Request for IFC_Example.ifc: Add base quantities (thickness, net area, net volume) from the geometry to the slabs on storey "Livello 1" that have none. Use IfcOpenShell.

First a look at what the model holds.

```python
import ifcopenshell
import ifcopenshell.util.element
import ifcopenshell.util.unit

model = ifcopenshell.open("IFC_Example.ifc")
print(model.schema)
for unit_type in ("LENGTHUNIT", "AREAUNIT", "VOLUMEUNIT"):
    print(unit_type, ifcopenshell.util.unit.calculate_unit_scale(model, unit_type))
storey = next(s for s in model.by_type("IfcBuildingStorey") if s.Name == "Livello 1")
slabs = [e for e in ifcopenshell.util.element.get_decomposition(storey) if e.is_a("IfcSlab")]
for e in sorted(slabs, key=lambda e: e.id()):
    print(e.id(), e.is_a(), e.Name, list(ifcopenshell.util.element.get_psets(e, qtos_only=True)), sep=" | ")
```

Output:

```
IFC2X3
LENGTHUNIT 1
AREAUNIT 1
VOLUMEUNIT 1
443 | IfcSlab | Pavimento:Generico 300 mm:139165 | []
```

```python
import ifcopenshell
import ifcopenshell.api.pset
import ifcopenshell.geom
import ifcopenshell.util.element
import ifcopenshell.util.shape
import ifcopenshell.util.unit

model = ifcopenshell.open("IFC_Example.ifc")
unit_scale = ifcopenshell.util.unit.calculate_unit_scale(model)
area_scale = ifcopenshell.util.unit.calculate_unit_scale(model, "AREAUNIT")
volume_scale = ifcopenshell.util.unit.calculate_unit_scale(model, "VOLUMEUNIT")
settings = ifcopenshell.geom.settings()

storey = next(s for s in model.by_type("IfcBuildingStorey") if s.Name == "Livello 1")
slabs = [e for e in ifcopenshell.util.element.get_decomposition(storey) if e.is_a("IfcSlab")]

for e in sorted(slabs, key=lambda e: e.id()):
    if ifcopenshell.util.element.get_psets(e, qtos_only=True, should_inherit=False):
        continue
    # Geometry comes back in metres, in the element's own axes.
    shape = ifcopenshell.geom.create_shape(settings, e)
    values = {
        "Width": ifcopenshell.util.shape.get_z(shape.geometry) / unit_scale,
        "NetArea": ifcopenshell.util.shape.get_footprint_area(shape.geometry) / area_scale,
        "NetVolume": ifcopenshell.util.shape.get_volume(shape.geometry) / volume_scale,
    }
    qto = ifcopenshell.api.pset.add_qto(model, product=e, name="BaseQuantities")
    ifcopenshell.api.pset.edit_qto(model, qto=qto, properties=values)
    print(e.id(), {k: round(v, 3) for k, v in values.items()})

model.write("IFC_Example_updated.ifc")
```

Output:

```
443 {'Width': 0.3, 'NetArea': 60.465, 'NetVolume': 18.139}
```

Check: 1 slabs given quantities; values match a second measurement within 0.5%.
